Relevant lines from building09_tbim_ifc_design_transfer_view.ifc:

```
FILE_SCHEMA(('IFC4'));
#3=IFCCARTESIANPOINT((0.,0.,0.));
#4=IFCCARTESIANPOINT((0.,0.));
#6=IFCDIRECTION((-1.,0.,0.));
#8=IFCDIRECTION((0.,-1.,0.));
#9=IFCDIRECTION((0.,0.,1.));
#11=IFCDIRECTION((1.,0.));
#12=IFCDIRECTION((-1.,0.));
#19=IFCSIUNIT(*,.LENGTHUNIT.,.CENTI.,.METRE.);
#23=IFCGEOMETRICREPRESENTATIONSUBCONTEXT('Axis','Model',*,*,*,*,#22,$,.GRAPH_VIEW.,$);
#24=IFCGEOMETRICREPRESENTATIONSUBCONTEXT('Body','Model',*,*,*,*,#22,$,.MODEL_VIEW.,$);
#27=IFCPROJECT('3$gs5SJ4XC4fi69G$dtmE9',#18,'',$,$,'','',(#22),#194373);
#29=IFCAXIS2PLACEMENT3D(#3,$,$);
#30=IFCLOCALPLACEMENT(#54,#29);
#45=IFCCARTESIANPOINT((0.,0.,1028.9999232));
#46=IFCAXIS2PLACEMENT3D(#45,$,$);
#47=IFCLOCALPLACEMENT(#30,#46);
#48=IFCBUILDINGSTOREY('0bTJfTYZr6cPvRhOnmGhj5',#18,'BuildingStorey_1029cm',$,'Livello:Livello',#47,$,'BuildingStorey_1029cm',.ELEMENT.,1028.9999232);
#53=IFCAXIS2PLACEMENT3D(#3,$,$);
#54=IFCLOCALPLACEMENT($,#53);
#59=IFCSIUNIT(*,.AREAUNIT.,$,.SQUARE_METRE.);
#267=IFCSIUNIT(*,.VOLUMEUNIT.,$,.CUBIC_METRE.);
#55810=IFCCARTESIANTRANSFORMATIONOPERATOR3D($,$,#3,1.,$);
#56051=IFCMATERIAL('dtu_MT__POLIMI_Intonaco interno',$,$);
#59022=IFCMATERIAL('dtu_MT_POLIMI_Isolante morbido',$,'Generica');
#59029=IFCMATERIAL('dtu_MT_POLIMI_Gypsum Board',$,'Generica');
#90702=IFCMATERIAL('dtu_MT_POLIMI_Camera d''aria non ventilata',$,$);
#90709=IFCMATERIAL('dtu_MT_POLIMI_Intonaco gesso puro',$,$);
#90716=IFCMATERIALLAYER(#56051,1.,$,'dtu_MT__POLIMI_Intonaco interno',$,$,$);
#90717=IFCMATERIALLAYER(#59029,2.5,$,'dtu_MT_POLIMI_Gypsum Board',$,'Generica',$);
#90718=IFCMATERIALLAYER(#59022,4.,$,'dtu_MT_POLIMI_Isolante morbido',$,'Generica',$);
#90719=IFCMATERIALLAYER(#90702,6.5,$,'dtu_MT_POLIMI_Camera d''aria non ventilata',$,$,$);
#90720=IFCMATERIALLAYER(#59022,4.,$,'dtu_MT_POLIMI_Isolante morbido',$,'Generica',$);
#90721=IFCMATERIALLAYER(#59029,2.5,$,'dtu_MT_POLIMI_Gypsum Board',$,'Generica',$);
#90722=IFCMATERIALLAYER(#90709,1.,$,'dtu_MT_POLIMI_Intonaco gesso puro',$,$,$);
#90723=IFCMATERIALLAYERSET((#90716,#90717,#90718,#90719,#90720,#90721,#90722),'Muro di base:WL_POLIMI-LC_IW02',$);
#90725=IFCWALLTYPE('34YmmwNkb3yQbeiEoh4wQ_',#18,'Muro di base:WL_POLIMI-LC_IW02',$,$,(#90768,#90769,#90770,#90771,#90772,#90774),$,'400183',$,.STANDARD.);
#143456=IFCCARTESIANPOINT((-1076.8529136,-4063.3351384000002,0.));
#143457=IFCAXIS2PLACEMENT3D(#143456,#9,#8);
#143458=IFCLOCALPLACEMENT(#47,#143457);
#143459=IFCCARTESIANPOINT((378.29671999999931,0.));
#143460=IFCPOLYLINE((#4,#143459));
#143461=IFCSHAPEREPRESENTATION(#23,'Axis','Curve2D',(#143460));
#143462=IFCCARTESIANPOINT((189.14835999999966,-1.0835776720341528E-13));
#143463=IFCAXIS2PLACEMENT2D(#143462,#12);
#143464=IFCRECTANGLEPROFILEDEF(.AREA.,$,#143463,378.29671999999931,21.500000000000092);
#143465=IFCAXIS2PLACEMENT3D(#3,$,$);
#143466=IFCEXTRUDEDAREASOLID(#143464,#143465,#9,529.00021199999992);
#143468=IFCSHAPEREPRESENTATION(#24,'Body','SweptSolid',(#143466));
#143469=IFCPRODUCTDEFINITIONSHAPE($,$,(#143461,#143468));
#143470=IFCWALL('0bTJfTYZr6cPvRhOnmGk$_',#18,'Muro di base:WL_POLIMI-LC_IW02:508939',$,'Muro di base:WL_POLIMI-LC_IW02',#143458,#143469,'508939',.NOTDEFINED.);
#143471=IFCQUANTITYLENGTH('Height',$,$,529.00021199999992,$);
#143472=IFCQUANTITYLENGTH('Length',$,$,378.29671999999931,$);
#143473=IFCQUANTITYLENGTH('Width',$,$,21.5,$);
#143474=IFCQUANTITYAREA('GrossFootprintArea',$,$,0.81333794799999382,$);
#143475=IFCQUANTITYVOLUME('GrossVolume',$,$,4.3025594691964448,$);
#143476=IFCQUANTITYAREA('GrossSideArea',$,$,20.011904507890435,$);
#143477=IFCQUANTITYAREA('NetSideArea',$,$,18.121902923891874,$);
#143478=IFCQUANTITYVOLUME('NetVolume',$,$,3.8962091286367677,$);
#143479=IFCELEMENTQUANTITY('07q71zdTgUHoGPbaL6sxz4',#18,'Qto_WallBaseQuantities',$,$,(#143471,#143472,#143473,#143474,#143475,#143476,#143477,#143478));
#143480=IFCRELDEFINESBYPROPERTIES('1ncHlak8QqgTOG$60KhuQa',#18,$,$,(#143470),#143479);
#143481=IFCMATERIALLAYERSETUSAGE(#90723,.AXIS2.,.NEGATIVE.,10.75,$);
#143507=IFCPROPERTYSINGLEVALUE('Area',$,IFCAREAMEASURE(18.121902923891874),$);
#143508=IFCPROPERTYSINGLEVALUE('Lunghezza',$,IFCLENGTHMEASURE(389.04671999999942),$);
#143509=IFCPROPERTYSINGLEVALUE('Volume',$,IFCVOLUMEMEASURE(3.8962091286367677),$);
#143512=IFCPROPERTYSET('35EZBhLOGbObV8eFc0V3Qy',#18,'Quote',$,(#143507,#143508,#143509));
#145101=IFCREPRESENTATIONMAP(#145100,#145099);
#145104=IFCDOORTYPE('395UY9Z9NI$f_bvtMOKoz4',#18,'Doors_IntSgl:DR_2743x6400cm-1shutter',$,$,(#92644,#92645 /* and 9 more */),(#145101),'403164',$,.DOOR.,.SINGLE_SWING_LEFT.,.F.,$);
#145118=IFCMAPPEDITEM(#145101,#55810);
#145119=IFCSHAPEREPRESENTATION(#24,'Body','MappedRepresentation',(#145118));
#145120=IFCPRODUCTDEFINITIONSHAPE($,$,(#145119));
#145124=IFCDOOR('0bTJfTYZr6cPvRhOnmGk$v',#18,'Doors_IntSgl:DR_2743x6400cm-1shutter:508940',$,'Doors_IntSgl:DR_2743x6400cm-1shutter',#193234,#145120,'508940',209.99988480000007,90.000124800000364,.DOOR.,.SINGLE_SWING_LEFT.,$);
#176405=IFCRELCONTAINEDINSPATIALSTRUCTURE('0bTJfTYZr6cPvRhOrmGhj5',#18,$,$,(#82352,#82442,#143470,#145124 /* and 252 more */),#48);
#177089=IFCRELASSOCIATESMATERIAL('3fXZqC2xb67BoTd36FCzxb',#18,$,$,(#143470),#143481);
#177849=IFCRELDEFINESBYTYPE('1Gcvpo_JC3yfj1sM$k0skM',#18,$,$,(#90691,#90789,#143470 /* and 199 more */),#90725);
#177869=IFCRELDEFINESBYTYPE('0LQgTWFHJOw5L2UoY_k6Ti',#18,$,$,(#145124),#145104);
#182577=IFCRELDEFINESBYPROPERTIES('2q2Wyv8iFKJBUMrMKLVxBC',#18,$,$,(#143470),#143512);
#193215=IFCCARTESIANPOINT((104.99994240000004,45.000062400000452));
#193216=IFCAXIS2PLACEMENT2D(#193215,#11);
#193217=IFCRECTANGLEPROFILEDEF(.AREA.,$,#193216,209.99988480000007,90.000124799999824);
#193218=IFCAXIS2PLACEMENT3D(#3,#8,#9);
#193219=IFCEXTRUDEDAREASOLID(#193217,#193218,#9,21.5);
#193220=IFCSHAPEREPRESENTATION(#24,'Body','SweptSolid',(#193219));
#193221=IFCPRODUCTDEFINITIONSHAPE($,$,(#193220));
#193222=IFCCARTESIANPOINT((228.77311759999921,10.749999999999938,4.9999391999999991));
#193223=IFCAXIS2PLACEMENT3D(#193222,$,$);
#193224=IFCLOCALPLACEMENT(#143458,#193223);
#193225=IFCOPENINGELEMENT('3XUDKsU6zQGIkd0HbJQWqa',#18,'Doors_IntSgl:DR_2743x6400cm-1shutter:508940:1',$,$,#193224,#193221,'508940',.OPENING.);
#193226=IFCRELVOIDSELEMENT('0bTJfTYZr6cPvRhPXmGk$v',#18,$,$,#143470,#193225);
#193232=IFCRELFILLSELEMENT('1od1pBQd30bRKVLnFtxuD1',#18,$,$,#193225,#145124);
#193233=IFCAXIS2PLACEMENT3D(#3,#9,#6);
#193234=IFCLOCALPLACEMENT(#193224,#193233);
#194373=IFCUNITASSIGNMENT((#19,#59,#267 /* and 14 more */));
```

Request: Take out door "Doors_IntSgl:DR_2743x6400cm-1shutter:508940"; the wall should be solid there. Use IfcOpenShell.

```python
import ifcopenshell
import ifcopenshell.api.feature
import ifcopenshell.api.pset
import ifcopenshell.api.root
import ifcopenshell.geom
import ifcopenshell.util.element
import ifcopenshell.util.shape
import ifcopenshell.util.unit

model = ifcopenshell.open("building09_tbim_ifc_design_transfer_view.ifc")
area_scale = ifcopenshell.util.unit.calculate_unit_scale(model, "AREAUNIT")
volume_scale = ifcopenshell.util.unit.calculate_unit_scale(model, "VOLUMEUNIT")
settings = ifcopenshell.geom.settings()


def volume(element):
    """Net volume in cubic metres, openings subtracted."""
    shape = ifcopenshell.geom.create_shape(settings, element)
    return ifcopenshell.util.shape.get_volume(shape.geometry)


door = model.by_guid("0bTJfTYZr6cPvRhOnmGk$v")
opening = door.FillsVoids[0].RelatingOpeningElement
wall = opening.VoidsElements[0].RelatingBuildingElement
before = volume(wall)

ifcopenshell.api.root.remove_product(model, product=door)
ifcopenshell.api.feature.remove_feature(model, feature=opening)

after = volume(wall)
thickness = 0.215  # wall thickness in metres

# Update the wall's stored quantities.
qto = model.by_id(ifcopenshell.util.element.get_pset(wall, "Qto_WallBaseQuantities", should_inherit=False)["id"])
ifcopenshell.api.pset.edit_qto(model, qto=qto, properties={
    "NetSideArea": after / thickness / area_scale,
    "NetVolume": after / volume_scale,
})
pset = model.by_id(ifcopenshell.util.element.get_pset(wall, "Quote", should_inherit=False)["id"])
ifcopenshell.api.pset.edit_pset(model, pset=pset, properties={
    "Area": model.create_entity("IfcAreaMeasure", after / thickness / area_scale),
    "Volume": model.create_entity("IfcVolumeMeasure", after / volume_scale),
})

print(f"wall volume {before:.3f} -> {after:.3f} m3")

model.write("building09_tbim_ifc_design_transfer_view_rev.ifc")
```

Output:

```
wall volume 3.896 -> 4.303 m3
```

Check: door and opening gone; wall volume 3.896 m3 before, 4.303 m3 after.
